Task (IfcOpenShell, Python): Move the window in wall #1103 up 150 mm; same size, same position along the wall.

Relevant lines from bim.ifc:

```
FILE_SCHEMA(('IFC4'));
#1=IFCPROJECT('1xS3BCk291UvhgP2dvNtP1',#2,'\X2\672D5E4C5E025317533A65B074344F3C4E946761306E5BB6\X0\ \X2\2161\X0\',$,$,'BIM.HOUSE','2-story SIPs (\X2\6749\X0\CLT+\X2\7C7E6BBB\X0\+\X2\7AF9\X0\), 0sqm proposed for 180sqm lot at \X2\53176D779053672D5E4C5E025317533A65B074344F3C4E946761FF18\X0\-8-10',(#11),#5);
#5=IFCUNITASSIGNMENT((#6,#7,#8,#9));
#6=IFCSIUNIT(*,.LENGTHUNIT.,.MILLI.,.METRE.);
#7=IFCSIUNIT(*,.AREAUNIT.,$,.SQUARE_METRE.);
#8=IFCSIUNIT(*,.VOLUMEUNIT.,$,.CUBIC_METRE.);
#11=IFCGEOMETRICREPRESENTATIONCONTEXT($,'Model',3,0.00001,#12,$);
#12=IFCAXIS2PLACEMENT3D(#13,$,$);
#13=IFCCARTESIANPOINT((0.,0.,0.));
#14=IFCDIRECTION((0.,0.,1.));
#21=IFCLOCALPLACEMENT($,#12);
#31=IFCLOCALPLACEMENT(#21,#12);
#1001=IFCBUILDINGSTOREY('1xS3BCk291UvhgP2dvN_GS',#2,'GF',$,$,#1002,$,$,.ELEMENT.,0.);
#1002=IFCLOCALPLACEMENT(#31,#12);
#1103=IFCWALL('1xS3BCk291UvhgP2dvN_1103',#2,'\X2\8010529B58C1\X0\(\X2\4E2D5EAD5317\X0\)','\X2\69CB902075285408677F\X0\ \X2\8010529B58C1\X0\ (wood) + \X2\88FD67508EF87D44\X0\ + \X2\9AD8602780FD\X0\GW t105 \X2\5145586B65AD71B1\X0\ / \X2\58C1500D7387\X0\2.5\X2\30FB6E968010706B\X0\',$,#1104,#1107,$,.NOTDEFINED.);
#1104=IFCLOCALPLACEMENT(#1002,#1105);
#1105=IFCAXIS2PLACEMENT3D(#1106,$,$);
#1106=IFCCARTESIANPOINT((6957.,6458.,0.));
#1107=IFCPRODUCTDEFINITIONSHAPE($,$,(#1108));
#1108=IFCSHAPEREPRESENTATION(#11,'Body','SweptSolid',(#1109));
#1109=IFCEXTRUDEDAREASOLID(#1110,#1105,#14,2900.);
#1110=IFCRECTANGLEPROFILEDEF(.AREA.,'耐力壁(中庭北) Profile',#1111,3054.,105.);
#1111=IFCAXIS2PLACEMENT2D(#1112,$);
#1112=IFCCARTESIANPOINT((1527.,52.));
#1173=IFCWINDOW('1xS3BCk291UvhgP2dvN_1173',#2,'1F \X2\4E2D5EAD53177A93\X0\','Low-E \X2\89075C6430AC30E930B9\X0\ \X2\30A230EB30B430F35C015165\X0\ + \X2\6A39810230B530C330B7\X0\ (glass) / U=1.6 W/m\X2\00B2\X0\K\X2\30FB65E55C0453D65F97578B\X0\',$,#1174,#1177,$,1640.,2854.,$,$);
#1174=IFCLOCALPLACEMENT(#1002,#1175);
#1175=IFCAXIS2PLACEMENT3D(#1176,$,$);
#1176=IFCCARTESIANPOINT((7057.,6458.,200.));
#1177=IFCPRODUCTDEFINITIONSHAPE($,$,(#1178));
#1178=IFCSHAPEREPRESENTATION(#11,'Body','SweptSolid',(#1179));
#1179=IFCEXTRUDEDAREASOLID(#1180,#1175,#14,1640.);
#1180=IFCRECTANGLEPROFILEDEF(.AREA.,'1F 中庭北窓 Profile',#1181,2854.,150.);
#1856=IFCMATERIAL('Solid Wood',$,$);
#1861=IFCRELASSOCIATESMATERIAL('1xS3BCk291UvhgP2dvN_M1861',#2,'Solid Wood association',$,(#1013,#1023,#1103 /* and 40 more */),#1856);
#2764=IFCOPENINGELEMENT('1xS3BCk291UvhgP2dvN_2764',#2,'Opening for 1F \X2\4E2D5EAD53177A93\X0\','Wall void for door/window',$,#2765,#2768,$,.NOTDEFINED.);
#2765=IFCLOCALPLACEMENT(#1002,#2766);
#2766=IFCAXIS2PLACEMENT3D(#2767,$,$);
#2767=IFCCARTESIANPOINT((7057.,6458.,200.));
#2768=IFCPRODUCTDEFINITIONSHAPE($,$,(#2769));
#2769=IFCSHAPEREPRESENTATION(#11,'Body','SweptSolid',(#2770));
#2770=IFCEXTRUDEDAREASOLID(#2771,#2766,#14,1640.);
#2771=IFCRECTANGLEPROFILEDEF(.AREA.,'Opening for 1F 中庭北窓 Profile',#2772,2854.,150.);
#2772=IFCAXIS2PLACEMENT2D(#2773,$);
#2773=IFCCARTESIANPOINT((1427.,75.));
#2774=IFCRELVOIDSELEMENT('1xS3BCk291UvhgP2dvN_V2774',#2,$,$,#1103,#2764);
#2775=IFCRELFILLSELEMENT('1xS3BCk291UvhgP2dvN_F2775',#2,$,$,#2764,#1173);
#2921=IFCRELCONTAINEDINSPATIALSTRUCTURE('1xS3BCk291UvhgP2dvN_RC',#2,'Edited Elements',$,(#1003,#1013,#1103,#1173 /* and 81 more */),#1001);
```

```python
import numpy as np
import ifcopenshell
import ifcopenshell.api.geometry
import ifcopenshell.util.placement
import ifcopenshell.util.unit

model = ifcopenshell.open("bim.ifc")
unit_scale = ifcopenshell.util.unit.calculate_unit_scale(model)

window = model.by_guid("1xS3BCk291UvhgP2dvN_1173")
opening = window.FillsVoids[0].RelatingOpeningElement
dz = 0.15 / unit_scale

shift = np.array([0.0, 0.0, dz])
# The window is not placed relative to its opening, so move both.
for product in (opening, window):
    matrix = ifcopenshell.util.placement.get_local_placement(product.ObjectPlacement)
    matrix[:3, 3] += shift
    ifcopenshell.api.geometry.edit_object_placement(model, product=product, matrix=matrix, is_si=False)

print(f"moved by {dz * unit_scale:+.3f} m")

model.write("bim_rev.ifc")
```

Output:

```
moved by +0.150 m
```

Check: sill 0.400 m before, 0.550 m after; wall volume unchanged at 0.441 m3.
